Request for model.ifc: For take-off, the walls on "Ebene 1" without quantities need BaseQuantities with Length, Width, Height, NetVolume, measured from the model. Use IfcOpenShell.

First a look at what the model holds.

```python
import ifcopenshell
import ifcopenshell.util.element
import ifcopenshell.util.unit

model = ifcopenshell.open("model.ifc")
print(model.schema)
for unit_type in ("LENGTHUNIT", "AREAUNIT", "VOLUMEUNIT"):
    print(unit_type, ifcopenshell.util.unit.calculate_unit_scale(model, unit_type))
storey = next(s for s in model.by_type("IfcBuildingStorey") if s.Name == "Ebene 1")
walls = [e for e in ifcopenshell.util.element.get_decomposition(storey) if e.is_a("IfcWall")]
for e in sorted(walls, key=lambda e: e.id()):
    print(e.id(), e.is_a(), e.Name, list(ifcopenshell.util.element.get_psets(e, qtos_only=True)), sep=" | ")
```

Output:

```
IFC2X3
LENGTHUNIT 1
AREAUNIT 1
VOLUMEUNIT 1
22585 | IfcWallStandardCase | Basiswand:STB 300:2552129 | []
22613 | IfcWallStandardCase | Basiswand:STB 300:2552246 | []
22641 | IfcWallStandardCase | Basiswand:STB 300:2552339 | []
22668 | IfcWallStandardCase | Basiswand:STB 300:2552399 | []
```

```python
import ifcopenshell
import ifcopenshell.api.pset
import ifcopenshell.geom
import ifcopenshell.util.element
import ifcopenshell.util.shape
import ifcopenshell.util.unit

model = ifcopenshell.open("model.ifc")
unit_scale = ifcopenshell.util.unit.calculate_unit_scale(model)
volume_scale = ifcopenshell.util.unit.calculate_unit_scale(model, "VOLUMEUNIT")
settings = ifcopenshell.geom.settings()

storey = next(s for s in model.by_type("IfcBuildingStorey") if s.Name == "Ebene 1")
walls = [e for e in ifcopenshell.util.element.get_decomposition(storey) if e.is_a("IfcWall")]

for e in sorted(walls, key=lambda e: e.id()):
    if ifcopenshell.util.element.get_psets(e, qtos_only=True, should_inherit=False):
        continue
    # Geometry comes back in metres, in the element's own axes.
    shape = ifcopenshell.geom.create_shape(settings, e)
    values = {
        "Length": ifcopenshell.util.shape.get_x(shape.geometry) / unit_scale,
        "Width": ifcopenshell.util.shape.get_y(shape.geometry) / unit_scale,
        "Height": ifcopenshell.util.shape.get_z(shape.geometry) / unit_scale,
        "NetVolume": ifcopenshell.util.shape.get_volume(shape.geometry) / volume_scale,
    }
    qto = ifcopenshell.api.pset.add_qto(model, product=e, name="BaseQuantities")
    ifcopenshell.api.pset.edit_qto(model, qto=qto, properties=values)
    print(e.id(), {k: round(v, 3) for k, v in values.items()})

model.write("model_rev.ifc")
```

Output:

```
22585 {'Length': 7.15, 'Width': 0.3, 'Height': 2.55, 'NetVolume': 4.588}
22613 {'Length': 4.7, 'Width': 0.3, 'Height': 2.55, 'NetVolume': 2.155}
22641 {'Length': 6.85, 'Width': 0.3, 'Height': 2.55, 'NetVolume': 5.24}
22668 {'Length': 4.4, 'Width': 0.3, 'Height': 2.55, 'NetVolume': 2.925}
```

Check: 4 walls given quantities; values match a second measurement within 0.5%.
